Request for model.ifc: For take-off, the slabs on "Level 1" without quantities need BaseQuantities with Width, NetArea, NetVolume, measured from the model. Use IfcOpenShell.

First a look at what the model holds.

```python
import ifcopenshell
import ifcopenshell.util.element
import ifcopenshell.util.unit

model = ifcopenshell.open("model.ifc")
print(model.schema)
for unit_type in ("LENGTHUNIT", "AREAUNIT", "VOLUMEUNIT"):
    print(unit_type, ifcopenshell.util.unit.calculate_unit_scale(model, unit_type))
storey = next(s for s in model.by_type("IfcBuildingStorey") if s.Name == "Level 1")
slabs = [e for e in ifcopenshell.util.element.get_decomposition(storey) if e.is_a("IfcSlab")]
for e in sorted(slabs, key=lambda e: e.id()):
    print(e.id(), e.is_a(), e.Name, list(ifcopenshell.util.element.get_psets(e, qtos_only=True)), sep=" | ")
```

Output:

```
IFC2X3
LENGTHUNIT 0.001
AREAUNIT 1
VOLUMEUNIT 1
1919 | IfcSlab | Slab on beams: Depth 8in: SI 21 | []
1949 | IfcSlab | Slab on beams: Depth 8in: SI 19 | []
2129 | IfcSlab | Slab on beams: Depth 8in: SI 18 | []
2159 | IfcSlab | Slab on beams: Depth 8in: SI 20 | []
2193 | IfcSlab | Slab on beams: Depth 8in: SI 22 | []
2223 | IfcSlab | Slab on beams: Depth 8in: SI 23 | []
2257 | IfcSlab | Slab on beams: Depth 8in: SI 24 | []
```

```python
import ifcopenshell
import ifcopenshell.api.pset
import ifcopenshell.geom
import ifcopenshell.util.element
import ifcopenshell.util.shape
import ifcopenshell.util.unit

model = ifcopenshell.open("model.ifc")
unit_scale = ifcopenshell.util.unit.calculate_unit_scale(model)
area_scale = ifcopenshell.util.unit.calculate_unit_scale(model, "AREAUNIT")
volume_scale = ifcopenshell.util.unit.calculate_unit_scale(model, "VOLUMEUNIT")
settings = ifcopenshell.geom.settings()

storey = next(s for s in model.by_type("IfcBuildingStorey") if s.Name == "Level 1")
slabs = [e for e in ifcopenshell.util.element.get_decomposition(storey) if e.is_a("IfcSlab")]

for e in sorted(slabs, key=lambda e: e.id()):
    if ifcopenshell.util.element.get_psets(e, qtos_only=True, should_inherit=False):
        continue
    # Geometry comes back in metres, in the element's own axes.
    shape = ifcopenshell.geom.create_shape(settings, e)
    values = {
        "Width": ifcopenshell.util.shape.get_z(shape.geometry) / unit_scale,
        "NetArea": ifcopenshell.util.shape.get_footprint_area(shape.geometry) / area_scale,
        "NetVolume": ifcopenshell.util.shape.get_volume(shape.geometry) / volume_scale,
    }
    qto = ifcopenshell.api.pset.add_qto(model, product=e, name="BaseQuantities")
    ifcopenshell.api.pset.edit_qto(model, qto=qto, properties=values)
    print(e.id(), {k: round(v, 3) for k, v in values.items()})

model.write("model-out.ifc")
```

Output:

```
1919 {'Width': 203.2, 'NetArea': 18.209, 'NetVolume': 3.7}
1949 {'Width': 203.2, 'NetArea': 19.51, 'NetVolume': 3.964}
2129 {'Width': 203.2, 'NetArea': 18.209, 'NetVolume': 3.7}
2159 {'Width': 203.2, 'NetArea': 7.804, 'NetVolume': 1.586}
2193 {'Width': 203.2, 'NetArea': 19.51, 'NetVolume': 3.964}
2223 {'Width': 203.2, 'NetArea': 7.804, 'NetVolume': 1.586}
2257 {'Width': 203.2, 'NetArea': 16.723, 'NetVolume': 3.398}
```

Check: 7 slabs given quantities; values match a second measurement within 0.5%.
